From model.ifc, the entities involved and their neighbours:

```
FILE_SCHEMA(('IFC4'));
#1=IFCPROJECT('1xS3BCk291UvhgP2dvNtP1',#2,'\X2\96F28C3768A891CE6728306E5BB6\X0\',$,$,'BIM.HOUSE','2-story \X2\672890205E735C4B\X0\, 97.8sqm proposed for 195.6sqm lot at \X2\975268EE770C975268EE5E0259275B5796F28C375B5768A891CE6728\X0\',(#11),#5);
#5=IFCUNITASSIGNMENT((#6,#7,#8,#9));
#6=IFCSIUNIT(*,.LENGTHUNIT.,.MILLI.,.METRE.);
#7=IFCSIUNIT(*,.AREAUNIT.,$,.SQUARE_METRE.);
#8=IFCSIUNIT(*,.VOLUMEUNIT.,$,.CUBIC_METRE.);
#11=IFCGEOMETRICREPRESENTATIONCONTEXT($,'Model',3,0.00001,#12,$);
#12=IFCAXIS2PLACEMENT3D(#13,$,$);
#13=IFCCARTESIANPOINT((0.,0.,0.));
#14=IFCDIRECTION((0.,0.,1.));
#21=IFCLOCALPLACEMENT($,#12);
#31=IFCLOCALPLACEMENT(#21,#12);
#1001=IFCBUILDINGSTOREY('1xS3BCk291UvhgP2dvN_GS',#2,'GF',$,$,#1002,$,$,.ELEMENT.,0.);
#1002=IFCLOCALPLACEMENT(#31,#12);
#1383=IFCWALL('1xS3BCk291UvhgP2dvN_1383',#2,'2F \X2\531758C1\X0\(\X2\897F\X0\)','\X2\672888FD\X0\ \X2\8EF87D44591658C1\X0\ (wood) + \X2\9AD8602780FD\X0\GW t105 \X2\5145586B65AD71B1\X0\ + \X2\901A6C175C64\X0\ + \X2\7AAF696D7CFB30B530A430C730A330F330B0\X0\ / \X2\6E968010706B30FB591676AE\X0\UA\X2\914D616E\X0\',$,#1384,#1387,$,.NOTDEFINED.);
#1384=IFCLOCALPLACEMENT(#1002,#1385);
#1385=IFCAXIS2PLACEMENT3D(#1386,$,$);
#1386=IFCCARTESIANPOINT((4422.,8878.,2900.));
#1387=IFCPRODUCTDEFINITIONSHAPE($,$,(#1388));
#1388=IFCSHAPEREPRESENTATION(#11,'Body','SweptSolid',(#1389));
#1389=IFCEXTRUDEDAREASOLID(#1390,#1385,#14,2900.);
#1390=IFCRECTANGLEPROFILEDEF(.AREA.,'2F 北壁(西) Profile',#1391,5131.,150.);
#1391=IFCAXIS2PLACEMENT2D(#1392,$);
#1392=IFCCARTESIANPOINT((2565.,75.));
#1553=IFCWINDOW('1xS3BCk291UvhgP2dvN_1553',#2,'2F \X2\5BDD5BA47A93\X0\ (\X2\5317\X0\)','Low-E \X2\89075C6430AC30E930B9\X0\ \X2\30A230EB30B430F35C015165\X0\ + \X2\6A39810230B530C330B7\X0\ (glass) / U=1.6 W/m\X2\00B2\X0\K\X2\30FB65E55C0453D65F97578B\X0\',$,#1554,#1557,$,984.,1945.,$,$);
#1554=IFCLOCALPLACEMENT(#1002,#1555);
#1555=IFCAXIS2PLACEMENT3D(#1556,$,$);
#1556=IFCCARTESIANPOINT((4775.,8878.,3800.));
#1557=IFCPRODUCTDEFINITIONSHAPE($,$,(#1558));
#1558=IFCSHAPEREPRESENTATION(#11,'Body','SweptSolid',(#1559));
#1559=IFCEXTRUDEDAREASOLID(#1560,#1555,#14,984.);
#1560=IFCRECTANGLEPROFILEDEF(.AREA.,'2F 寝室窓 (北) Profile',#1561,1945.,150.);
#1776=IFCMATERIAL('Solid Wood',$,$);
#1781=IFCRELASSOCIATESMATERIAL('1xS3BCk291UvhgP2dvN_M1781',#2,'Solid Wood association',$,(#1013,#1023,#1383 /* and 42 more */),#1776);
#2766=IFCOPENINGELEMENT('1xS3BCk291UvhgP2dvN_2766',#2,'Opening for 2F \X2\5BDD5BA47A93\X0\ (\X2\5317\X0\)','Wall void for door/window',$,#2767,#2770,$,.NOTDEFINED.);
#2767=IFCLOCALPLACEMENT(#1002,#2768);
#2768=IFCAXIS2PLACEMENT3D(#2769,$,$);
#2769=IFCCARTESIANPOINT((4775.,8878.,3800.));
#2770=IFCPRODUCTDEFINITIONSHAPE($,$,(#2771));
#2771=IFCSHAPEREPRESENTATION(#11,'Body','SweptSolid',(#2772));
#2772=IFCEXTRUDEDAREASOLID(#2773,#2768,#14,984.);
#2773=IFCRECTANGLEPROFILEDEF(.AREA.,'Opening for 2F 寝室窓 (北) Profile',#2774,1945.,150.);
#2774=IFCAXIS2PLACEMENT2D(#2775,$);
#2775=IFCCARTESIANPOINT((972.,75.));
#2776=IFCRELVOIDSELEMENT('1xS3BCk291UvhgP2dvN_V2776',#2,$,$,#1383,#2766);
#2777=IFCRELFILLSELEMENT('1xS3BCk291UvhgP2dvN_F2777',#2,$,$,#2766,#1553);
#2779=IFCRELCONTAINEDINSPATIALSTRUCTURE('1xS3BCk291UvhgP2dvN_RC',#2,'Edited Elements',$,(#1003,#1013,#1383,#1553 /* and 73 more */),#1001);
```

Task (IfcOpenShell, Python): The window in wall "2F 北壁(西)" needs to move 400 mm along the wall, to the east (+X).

```python
import ifcopenshell
import ifcopenshell.api.geometry
import ifcopenshell.util.placement
import ifcopenshell.util.unit

model = ifcopenshell.open("model.ifc")
unit_scale = ifcopenshell.util.unit.calculate_unit_scale(model)

window = model.by_id(1553)
opening = window.FillsVoids[0].RelatingOpeningElement
wall = opening.VoidsElements[0].RelatingBuildingElement

wall_matrix = ifcopenshell.util.placement.get_local_placement(wall.ObjectPlacement)
shift = wall_matrix[:3, 0] * 0.4 / unit_scale
before = ifcopenshell.util.placement.get_local_placement(window.ObjectPlacement)[:3, 3].copy()

# The window is not placed relative to its opening, so move both.
for product in (opening, window):
    matrix = ifcopenshell.util.placement.get_local_placement(product.ObjectPlacement)
    matrix[:3, 3] += shift
    ifcopenshell.api.geometry.edit_object_placement(model, product=product, matrix=matrix, is_si=False)

after = ifcopenshell.util.placement.get_local_placement(window.ObjectPlacement)[:3, 3]
print("window moved by", (after - before).round(3) + 0.0)

model.write("model_v2.ifc")
```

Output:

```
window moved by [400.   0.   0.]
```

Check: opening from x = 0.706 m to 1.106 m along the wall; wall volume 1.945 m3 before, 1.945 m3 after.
